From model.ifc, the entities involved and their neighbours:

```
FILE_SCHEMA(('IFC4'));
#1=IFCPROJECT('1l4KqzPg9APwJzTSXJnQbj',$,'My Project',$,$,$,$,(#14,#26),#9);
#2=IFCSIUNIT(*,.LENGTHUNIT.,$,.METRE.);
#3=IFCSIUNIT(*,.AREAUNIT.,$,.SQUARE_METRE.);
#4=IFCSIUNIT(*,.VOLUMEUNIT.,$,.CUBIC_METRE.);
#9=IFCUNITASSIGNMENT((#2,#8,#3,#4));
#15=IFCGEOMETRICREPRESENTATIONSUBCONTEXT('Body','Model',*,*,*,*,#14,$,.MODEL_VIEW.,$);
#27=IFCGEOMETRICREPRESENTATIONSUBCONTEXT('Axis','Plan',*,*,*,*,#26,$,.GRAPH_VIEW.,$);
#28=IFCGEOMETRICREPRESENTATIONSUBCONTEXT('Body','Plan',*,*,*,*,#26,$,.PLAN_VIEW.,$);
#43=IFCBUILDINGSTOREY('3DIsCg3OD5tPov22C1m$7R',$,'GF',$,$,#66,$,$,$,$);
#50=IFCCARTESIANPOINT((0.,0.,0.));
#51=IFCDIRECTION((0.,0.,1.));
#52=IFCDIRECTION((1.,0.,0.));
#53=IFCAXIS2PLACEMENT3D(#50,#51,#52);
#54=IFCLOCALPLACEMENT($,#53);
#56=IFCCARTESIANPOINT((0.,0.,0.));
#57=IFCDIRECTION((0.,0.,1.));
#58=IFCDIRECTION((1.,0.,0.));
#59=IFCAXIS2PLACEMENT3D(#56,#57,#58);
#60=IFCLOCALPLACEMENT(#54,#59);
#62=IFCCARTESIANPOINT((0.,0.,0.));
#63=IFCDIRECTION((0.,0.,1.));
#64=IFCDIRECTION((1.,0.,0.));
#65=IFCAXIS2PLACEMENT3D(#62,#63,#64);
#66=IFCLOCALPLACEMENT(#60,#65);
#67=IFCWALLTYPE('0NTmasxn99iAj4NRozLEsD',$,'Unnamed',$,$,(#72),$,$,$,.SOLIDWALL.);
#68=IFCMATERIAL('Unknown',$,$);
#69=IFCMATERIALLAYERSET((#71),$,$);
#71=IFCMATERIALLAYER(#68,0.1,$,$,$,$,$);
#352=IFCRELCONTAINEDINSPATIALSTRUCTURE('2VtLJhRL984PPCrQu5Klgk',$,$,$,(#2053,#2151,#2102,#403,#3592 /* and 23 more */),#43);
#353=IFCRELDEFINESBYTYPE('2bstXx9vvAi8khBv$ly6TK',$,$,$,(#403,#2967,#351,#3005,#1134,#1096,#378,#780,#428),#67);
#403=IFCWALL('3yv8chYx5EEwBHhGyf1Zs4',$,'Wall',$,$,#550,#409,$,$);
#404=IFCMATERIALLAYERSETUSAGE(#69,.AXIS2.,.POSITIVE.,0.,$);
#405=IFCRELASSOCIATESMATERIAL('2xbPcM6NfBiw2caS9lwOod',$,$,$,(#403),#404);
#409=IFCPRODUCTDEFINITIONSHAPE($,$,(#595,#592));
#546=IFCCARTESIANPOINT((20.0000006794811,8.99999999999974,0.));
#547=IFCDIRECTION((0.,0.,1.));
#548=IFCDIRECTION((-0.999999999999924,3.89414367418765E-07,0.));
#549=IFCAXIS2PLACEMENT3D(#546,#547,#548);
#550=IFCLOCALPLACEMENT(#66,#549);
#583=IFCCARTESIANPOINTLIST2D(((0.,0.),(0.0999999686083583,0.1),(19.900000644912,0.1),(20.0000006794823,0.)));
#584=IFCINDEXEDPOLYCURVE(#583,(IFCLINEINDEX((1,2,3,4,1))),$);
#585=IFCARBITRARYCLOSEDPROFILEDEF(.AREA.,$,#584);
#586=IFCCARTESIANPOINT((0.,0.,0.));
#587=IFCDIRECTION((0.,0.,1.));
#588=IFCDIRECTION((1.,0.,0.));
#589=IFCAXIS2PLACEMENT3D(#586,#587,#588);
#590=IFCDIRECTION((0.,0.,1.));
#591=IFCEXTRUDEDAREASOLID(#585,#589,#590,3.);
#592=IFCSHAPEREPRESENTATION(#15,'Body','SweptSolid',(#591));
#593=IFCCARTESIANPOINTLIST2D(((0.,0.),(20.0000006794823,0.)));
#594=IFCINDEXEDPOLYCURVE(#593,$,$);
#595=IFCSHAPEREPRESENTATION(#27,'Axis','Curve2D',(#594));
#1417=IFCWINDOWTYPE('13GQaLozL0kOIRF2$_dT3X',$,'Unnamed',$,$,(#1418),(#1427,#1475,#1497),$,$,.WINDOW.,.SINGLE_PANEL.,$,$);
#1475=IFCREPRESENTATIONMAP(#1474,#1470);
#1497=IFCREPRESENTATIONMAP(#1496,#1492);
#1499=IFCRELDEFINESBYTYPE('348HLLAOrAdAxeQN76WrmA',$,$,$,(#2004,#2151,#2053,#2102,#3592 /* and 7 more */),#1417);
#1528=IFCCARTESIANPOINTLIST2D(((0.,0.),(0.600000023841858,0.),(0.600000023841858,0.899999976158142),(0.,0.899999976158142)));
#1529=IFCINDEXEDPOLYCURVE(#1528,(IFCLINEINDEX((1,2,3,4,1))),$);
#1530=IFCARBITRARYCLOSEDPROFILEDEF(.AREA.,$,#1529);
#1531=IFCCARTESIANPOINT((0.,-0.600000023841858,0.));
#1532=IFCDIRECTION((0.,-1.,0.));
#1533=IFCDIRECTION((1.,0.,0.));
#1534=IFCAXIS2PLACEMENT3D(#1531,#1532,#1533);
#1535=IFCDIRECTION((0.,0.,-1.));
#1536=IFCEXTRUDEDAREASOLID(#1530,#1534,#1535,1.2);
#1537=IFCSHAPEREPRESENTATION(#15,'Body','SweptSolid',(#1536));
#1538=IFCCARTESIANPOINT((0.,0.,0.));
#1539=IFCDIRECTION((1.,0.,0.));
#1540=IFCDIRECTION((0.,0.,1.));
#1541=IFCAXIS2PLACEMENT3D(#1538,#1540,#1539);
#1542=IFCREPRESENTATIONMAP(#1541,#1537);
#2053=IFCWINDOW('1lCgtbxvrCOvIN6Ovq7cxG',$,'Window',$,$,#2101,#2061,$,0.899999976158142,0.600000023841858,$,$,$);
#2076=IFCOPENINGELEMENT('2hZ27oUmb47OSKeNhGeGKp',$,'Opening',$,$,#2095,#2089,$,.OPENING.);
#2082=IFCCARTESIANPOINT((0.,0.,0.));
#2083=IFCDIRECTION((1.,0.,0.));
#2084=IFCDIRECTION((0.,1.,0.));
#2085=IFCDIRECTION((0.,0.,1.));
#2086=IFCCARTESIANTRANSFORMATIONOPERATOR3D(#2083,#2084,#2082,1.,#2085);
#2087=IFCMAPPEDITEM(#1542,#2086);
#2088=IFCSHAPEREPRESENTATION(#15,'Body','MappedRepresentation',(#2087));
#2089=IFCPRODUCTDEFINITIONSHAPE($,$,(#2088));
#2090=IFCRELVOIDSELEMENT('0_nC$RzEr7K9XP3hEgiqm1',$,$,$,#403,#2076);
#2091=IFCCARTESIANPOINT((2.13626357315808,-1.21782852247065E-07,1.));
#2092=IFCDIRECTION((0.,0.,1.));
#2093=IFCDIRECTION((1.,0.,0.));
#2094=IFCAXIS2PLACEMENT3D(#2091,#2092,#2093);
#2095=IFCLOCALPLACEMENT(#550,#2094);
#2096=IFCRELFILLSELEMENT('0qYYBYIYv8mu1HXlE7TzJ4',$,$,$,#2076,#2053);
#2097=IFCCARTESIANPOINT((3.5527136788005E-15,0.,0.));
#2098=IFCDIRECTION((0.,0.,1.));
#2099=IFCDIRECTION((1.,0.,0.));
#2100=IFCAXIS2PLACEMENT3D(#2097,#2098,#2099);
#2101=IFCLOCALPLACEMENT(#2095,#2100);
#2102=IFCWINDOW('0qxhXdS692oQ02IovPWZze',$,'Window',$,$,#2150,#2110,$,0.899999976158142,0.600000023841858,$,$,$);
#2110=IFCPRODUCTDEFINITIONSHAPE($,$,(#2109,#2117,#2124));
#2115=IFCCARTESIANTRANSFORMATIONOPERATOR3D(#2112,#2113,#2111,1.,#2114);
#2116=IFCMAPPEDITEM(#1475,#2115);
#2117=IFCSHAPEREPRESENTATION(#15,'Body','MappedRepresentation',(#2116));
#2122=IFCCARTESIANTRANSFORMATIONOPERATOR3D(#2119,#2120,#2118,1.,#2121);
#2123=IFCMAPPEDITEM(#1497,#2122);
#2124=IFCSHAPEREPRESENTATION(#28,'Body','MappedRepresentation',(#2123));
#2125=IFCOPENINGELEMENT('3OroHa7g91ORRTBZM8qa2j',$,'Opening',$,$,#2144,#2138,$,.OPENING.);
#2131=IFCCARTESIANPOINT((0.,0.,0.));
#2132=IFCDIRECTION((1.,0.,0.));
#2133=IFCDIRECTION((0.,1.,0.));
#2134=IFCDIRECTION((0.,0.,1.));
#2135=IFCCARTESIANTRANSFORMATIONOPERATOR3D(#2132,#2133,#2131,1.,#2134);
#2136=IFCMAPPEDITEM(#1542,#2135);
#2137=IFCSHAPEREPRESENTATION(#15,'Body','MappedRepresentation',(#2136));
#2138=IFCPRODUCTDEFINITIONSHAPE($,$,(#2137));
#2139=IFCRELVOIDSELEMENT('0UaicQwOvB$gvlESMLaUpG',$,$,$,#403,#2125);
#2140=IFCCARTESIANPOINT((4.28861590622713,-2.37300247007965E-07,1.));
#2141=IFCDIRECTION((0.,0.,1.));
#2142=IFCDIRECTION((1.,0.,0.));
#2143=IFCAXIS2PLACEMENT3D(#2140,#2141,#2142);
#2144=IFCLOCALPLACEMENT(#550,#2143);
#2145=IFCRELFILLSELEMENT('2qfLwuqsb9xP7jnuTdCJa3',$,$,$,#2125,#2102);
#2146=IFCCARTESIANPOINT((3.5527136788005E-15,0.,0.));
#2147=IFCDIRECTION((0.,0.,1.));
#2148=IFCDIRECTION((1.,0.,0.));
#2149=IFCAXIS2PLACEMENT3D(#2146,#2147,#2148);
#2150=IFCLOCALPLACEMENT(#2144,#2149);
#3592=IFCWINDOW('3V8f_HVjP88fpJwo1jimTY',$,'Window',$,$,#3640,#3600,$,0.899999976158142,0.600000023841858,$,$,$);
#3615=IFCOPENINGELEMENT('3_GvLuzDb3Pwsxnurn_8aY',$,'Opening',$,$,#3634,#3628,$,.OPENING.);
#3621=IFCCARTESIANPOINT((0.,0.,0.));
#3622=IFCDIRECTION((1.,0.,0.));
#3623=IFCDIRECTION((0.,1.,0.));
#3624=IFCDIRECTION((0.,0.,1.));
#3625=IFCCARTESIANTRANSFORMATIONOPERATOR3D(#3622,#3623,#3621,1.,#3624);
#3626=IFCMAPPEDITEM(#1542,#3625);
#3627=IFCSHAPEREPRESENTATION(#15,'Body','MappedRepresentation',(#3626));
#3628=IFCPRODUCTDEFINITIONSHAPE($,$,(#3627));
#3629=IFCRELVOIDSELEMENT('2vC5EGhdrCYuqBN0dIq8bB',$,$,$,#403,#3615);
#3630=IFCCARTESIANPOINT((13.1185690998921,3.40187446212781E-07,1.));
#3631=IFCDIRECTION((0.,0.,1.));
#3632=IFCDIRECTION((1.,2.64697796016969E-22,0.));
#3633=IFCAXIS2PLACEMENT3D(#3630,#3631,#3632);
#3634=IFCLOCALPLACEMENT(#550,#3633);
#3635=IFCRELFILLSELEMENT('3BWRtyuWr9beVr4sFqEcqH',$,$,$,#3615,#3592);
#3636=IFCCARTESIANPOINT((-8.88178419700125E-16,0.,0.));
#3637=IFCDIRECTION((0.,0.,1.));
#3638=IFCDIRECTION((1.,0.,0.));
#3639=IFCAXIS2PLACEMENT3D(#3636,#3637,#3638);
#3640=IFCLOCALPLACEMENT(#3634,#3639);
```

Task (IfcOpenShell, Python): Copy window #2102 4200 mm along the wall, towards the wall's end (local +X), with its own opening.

```python
import ifcopenshell
import ifcopenshell.api.feature
import ifcopenshell.api.geometry
import ifcopenshell.api.root
import ifcopenshell.geom
import ifcopenshell.util.element
import ifcopenshell.util.placement
import ifcopenshell.util.shape
import ifcopenshell.util.unit

model = ifcopenshell.open("model.ifc")
unit_scale = ifcopenshell.util.unit.calculate_unit_scale(model)
settings = ifcopenshell.geom.settings()


def volume(element):
    """Net volume in cubic metres, openings subtracted."""
    shape = ifcopenshell.geom.create_shape(settings, element)
    return ifcopenshell.util.shape.get_volume(shape.geometry)


window = model.by_guid("0qxhXdS692oQ02IovPWZze")
opening = window.FillsVoids[0].RelatingOpeningElement
wall = opening.VoidsElements[0].RelatingBuildingElement
before = volume(wall)
shift = ifcopenshell.util.placement.get_local_placement(wall.ObjectPlacement)[:3, 0] * 4.2 / unit_scale

# copy_class copies the void relationship, type, container and properties, but no geometry.
new_opening = ifcopenshell.api.root.copy_class(model, product=opening)
new_opening.Representation = ifcopenshell.util.element.copy_deep(
    model, opening.Representation, exclude=["IfcGeometricRepresentationContext", "IfcRepresentationMap"]
)
new_window = ifcopenshell.api.root.copy_class(model, product=window)
new_window.Representation = ifcopenshell.util.element.copy_deep(
    model, window.Representation, exclude=["IfcGeometricRepresentationContext", "IfcRepresentationMap"]
)
ifcopenshell.api.feature.add_filling(model, opening=new_opening, element=new_window)

for old, new in ((opening, new_opening), (window, new_window)):
    matrix = ifcopenshell.util.placement.get_local_placement(old.ObjectPlacement)
    matrix[:3, 3] += shift
    ifcopenshell.api.geometry.edit_object_placement(model, product=new, matrix=matrix, is_si=False)

after = volume(wall)

print(f"wall volume {before:.3f} -> {after:.3f} m3")

model.write("model_edited.ifc")
```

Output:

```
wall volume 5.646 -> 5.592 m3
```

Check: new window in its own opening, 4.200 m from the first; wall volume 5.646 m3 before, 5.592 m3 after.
